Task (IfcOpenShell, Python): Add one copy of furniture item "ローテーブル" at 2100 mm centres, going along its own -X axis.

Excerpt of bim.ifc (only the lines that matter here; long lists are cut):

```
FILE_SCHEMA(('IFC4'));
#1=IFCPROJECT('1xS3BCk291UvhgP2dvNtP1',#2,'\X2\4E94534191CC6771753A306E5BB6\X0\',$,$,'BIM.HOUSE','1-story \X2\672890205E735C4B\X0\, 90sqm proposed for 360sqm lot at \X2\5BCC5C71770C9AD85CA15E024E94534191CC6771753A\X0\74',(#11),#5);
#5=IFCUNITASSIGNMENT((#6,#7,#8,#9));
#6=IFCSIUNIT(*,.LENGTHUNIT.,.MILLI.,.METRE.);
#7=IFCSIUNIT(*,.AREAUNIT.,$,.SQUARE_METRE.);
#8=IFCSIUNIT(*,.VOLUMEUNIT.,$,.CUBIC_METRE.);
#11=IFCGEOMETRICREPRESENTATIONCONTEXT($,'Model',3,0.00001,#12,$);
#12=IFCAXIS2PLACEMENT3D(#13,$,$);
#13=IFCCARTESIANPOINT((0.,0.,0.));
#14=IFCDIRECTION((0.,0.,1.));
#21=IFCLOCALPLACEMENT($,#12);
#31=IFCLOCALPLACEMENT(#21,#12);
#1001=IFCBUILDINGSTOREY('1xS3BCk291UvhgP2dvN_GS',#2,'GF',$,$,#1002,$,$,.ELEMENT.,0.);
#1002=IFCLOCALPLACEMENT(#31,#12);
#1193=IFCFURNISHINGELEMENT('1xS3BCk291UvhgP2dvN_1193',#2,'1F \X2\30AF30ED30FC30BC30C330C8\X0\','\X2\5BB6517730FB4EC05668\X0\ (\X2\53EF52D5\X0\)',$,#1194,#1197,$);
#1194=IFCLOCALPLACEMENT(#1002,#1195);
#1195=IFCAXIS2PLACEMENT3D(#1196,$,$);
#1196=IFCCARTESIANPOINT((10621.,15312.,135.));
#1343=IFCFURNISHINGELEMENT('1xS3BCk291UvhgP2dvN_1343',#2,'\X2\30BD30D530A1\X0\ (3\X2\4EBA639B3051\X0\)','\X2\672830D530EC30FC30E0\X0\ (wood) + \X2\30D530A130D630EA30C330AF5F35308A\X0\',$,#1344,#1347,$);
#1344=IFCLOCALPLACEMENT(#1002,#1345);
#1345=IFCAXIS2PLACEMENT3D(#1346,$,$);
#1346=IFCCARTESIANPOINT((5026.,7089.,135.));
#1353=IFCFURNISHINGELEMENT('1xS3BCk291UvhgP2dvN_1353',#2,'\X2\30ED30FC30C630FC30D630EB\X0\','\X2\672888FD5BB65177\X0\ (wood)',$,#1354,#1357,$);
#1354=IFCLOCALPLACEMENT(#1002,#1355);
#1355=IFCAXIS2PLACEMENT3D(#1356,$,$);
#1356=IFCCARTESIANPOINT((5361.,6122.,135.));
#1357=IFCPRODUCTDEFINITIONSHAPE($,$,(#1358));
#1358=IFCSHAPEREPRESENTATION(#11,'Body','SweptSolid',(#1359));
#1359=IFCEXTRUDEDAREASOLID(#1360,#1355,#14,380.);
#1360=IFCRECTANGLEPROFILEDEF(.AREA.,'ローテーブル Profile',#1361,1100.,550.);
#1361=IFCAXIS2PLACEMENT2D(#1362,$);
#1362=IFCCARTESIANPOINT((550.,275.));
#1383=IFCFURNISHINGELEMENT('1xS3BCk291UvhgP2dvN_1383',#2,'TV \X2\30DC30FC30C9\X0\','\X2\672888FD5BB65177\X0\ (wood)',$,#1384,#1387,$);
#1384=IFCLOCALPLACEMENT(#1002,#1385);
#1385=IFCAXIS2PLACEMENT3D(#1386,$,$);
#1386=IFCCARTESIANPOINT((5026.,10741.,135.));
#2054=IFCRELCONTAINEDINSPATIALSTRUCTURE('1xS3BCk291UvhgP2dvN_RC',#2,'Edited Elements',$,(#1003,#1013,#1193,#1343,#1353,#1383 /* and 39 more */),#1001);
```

```python
import ifcopenshell
import ifcopenshell.api.geometry
import ifcopenshell.api.root
import ifcopenshell.util.element
import ifcopenshell.util.placement
import ifcopenshell.util.unit

model = ifcopenshell.open("bim.ifc")
unit_scale = ifcopenshell.util.unit.calculate_unit_scale(model)


def reuse_history(source, copy):
    """copy_class also copies each property set's owner history, people and application; keep the originals."""
    for rel in copy.IsDefinedBy:
        if rel.is_a("IfcRelDefinesByProperties") and (history := rel.RelatingPropertyDefinition.OwnerHistory):
            rel.RelatingPropertyDefinition.OwnerHistory = source.OwnerHistory
            ifcopenshell.util.element.remove_deep2(model, history)


source = model.by_guid("1xS3BCk291UvhgP2dvN_1353")
base = ifcopenshell.util.placement.get_local_placement(source.ObjectPlacement)
step = -base[:3, 0] * 2.1 / unit_scale

for i in range(1, 2):
    copy = ifcopenshell.api.root.copy_class(model, product=source)
    copy.Representation = ifcopenshell.util.element.copy_deep(
        model, source.Representation, exclude=["IfcGeometricRepresentationContext", "IfcRepresentationMap"]
    )
    reuse_history(source, copy)
    matrix = base.copy()
    matrix[:3, 3] += i * step
    print("added at", matrix[:3, 3].round(3) + 0.0)
    ifcopenshell.api.geometry.edit_object_placement(model, product=copy, matrix=matrix, is_si=False)

model.write("bim_edited.ifc")
```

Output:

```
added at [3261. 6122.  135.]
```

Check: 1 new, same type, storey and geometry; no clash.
